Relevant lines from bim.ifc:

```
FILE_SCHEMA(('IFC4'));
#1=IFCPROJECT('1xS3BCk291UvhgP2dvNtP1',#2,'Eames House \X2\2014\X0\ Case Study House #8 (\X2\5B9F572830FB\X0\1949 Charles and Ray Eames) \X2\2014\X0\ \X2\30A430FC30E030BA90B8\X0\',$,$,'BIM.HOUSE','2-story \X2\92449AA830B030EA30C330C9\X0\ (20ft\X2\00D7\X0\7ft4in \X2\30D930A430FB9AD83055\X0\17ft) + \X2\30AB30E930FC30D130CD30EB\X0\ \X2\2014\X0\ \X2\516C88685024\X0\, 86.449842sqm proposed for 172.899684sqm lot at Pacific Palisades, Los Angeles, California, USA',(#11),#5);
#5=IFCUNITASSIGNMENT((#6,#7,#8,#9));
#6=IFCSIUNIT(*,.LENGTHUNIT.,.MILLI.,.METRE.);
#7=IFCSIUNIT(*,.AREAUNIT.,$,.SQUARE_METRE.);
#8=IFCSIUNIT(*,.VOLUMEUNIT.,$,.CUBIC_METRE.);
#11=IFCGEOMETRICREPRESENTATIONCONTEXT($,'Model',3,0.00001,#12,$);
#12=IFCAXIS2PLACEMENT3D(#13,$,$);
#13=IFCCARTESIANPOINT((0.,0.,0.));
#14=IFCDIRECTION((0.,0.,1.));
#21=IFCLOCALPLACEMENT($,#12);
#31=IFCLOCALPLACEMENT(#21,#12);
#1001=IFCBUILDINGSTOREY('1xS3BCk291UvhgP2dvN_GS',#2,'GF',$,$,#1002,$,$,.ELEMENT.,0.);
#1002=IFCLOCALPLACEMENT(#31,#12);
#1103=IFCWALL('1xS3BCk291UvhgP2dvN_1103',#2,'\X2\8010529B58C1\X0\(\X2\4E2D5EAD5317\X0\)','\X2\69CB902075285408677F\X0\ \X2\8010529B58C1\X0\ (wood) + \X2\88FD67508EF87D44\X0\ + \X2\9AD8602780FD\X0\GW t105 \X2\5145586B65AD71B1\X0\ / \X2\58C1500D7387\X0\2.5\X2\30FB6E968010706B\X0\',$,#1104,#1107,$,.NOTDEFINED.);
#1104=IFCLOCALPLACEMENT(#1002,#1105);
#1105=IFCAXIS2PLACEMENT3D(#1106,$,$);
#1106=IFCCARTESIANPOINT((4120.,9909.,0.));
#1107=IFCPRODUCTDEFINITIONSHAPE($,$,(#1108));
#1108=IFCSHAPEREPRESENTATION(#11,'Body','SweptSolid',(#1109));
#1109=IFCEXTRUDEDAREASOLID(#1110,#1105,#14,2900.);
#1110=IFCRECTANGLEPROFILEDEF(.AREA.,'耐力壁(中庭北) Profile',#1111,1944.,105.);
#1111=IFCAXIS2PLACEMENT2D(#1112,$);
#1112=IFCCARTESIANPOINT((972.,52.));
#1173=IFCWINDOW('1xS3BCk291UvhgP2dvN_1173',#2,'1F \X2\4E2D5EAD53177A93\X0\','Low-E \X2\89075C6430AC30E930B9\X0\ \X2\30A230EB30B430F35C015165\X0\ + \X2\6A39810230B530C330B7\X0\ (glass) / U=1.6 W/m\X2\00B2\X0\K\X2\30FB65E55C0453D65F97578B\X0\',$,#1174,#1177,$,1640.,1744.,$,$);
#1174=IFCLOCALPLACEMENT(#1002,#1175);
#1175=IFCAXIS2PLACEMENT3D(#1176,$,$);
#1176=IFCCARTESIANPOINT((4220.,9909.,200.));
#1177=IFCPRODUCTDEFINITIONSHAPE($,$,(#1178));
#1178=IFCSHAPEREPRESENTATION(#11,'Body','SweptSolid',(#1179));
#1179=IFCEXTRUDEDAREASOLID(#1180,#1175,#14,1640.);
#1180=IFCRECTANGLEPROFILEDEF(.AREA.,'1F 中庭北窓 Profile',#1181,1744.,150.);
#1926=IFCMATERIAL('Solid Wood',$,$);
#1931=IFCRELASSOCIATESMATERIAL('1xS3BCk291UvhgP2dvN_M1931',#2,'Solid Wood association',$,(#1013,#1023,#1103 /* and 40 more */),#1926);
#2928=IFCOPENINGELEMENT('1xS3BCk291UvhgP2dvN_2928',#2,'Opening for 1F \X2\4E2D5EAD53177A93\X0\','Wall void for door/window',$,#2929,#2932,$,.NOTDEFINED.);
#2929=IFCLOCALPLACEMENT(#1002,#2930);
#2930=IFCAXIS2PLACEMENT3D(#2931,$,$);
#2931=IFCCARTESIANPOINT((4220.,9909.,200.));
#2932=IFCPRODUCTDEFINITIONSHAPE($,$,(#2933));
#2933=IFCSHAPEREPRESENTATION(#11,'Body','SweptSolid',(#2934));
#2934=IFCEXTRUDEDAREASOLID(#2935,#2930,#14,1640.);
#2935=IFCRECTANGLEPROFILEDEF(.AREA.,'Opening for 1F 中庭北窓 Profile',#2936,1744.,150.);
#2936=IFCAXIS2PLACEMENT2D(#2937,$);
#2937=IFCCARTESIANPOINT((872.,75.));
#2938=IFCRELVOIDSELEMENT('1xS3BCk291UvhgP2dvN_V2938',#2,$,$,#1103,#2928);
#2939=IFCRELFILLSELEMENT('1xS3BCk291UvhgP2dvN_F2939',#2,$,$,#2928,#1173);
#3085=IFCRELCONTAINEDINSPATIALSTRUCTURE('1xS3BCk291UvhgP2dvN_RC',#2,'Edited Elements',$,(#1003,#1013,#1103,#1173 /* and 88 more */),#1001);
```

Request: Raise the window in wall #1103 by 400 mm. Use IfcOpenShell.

```python
import numpy as np
import ifcopenshell
import ifcopenshell.api.geometry
import ifcopenshell.util.placement
import ifcopenshell.util.unit

model = ifcopenshell.open("bim.ifc")
unit_scale = ifcopenshell.util.unit.calculate_unit_scale(model)

window = model.by_id(1173)
opening = window.FillsVoids[0].RelatingOpeningElement
dz = 0.4 / unit_scale

shift = np.array([0.0, 0.0, dz])
# The window is not placed relative to its opening, so move both.
for product in (opening, window):
    matrix = ifcopenshell.util.placement.get_local_placement(product.ObjectPlacement)
    matrix[:3, 3] += shift
    ifcopenshell.api.geometry.edit_object_placement(model, product=product, matrix=matrix, is_si=False)

print(f"moved by {dz * unit_scale:+.3f} m")

model.write("bim_v2.ifc")
```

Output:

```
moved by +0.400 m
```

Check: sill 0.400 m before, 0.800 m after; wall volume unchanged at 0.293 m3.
